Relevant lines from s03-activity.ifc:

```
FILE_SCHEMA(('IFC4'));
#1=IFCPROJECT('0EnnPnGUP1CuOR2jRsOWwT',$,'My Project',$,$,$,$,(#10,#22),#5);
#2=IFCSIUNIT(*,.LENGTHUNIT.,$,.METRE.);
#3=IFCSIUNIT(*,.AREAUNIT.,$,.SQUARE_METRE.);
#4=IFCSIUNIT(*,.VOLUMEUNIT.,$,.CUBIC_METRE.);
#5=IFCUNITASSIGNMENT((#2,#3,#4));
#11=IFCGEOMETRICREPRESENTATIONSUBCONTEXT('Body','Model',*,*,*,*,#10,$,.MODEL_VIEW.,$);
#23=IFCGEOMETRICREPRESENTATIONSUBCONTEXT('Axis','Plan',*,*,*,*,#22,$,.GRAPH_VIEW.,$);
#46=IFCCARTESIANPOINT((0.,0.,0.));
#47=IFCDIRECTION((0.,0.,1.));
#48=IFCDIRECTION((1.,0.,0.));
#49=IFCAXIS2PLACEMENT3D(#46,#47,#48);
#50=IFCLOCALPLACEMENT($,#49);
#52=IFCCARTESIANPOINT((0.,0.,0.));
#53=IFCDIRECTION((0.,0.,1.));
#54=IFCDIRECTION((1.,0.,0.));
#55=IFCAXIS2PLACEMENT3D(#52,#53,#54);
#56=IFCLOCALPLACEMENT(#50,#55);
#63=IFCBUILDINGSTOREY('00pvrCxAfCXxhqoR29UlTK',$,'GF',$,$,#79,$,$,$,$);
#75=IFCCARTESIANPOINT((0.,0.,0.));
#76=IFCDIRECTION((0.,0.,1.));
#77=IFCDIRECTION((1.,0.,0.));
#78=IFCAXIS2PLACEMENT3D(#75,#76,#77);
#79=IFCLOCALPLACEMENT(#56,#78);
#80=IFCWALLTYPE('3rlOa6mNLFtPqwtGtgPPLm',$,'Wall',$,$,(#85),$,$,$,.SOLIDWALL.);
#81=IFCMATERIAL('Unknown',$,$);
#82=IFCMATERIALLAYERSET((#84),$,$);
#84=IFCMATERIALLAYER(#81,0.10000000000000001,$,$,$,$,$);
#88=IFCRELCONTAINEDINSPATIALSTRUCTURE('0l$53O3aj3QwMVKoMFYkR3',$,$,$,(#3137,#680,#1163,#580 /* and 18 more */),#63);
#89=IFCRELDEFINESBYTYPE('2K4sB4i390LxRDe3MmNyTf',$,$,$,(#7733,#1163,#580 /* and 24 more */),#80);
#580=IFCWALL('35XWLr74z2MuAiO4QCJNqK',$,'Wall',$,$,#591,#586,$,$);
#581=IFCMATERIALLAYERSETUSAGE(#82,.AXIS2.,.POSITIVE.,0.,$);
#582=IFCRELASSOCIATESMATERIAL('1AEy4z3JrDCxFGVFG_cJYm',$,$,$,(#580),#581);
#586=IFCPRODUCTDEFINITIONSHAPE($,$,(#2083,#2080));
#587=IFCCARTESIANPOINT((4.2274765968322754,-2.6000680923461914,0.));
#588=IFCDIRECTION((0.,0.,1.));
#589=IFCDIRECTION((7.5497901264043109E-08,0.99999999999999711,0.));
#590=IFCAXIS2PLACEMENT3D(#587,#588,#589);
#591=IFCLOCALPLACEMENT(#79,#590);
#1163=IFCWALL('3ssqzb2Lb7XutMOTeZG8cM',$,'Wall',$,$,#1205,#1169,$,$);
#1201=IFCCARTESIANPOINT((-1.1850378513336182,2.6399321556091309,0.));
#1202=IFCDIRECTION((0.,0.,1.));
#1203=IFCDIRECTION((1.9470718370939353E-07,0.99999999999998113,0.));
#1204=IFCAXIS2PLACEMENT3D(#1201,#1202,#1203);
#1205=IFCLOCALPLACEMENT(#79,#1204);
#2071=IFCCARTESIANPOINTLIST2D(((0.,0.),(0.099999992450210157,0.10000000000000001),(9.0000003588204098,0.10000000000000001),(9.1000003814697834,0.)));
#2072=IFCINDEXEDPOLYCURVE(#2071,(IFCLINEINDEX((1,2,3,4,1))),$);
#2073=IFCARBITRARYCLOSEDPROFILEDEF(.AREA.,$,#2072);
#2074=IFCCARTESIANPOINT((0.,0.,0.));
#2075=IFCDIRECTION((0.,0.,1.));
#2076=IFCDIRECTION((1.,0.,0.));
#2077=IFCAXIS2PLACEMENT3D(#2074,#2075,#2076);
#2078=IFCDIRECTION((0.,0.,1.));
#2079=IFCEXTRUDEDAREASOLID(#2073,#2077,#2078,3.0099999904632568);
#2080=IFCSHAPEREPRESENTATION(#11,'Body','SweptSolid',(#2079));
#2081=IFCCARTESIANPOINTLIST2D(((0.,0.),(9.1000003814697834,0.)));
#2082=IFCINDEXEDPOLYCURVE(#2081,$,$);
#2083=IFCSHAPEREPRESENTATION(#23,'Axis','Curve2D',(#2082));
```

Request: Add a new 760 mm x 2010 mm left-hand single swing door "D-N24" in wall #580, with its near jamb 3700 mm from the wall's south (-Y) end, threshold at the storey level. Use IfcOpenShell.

```python
import numpy as np
import ifcopenshell
import ifcopenshell.api.feature
import ifcopenshell.api.geometry
import ifcopenshell.api.root
import ifcopenshell.api.spatial
import ifcopenshell.geom
import ifcopenshell.util.element
import ifcopenshell.util.placement
import ifcopenshell.util.representation
import ifcopenshell.util.shape
import ifcopenshell.util.unit

model = ifcopenshell.open("s03-activity.ifc")
unit_scale = ifcopenshell.util.unit.calculate_unit_scale(model)
settings = ifcopenshell.geom.settings()


def volume(element):
    """Net volume in cubic metres, openings subtracted."""
    shape = ifcopenshell.geom.create_shape(settings, element)
    return ifcopenshell.util.shape.get_volume(shape.geometry)


wall = model.by_id(580)
storey = ifcopenshell.util.element.get_container(wall, ifc_class="IfcBuildingStorey")
context = ifcopenshell.util.representation.get_context(model, "Model", "Body", "MODEL_VIEW")
before = volume(wall)

width, height, from_end, sill = 0.76, 2.01, 3.7, 0.0  # metres

# The wall runs along its own X axis, and the end named is its -X end.
wall_shape = ifcopenshell.geom.create_shape(settings, wall)
x, y, z = ifcopenshell.util.shape.get_vertices(wall_shape.geometry).T
start = x.min() + from_end
face, thickness = float(y.min()), float(y.max() - y.min())
wall_matrix = ifcopenshell.util.placement.get_local_placement(wall.ObjectPlacement)
level = ifcopenshell.util.placement.get_local_placement(storey.ObjectPlacement)[2, 3]


def in_wall(x, y):
    """Placement at x, y metres in the wall's axes, at sill height."""
    matrix = wall_matrix.copy()
    matrix[:, 3] = wall_matrix @ np.array([x / unit_scale, y / unit_scale, 0.0, 1.0])
    matrix[2, 3] = level + sill / unit_scale
    return matrix


# Opening: a box that overshoots both wall faces by 50 mm.
opening = ifcopenshell.api.root.create_entity(model, ifc_class="IfcOpeningElement", predefined_type="OPENING")
box = ifcopenshell.api.geometry.add_wall_representation(
    model, context=context, length=width, height=height, thickness=thickness + 0.1
)
ifcopenshell.api.geometry.assign_representation(model, product=opening, representation=box)
ifcopenshell.api.geometry.edit_object_placement(model, product=opening, matrix=in_wall(start, face - 0.05), is_si=False)
ifcopenshell.api.feature.add_feature(model, feature=opening, element=wall)

door = ifcopenshell.api.root.create_entity(model, ifc_class="IfcDoor", name="D-N24", predefined_type="DOOR")
door.OverallWidth, door.OverallHeight = width / unit_scale, height / unit_scale
door.OperationType = "SINGLE_SWING_LEFT"
body = ifcopenshell.api.geometry.add_door_representation(
    model,
    context=context,
    overall_width=door.OverallWidth,
    overall_height=door.OverallHeight,
    operation_type="SINGLE_SWING_LEFT",
    lining_properties={"LiningDepth": thickness / unit_scale, "ThresholdDepth": thickness / unit_scale},
)
ifcopenshell.api.geometry.assign_representation(model, product=door, representation=body)
ifcopenshell.api.spatial.assign_container(model, products=[door], relating_structure=storey)
ifcopenshell.api.feature.add_filling(model, opening=opening, element=door)

# The lining spans the wall, so the door starts at the wall face.
ifcopenshell.api.geometry.edit_object_placement(model, product=door, matrix=in_wall(start, face), is_si=False)

after = volume(wall)

print(f"wall volume {before:.3f} -> {after:.3f} m3")

model.write("s03-activity_v2.ifc")
```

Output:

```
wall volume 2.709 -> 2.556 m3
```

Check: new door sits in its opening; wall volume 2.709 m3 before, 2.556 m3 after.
